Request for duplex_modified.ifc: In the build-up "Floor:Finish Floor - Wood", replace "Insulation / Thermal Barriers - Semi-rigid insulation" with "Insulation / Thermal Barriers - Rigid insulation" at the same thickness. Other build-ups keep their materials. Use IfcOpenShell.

First a look at what the model holds.

```python
import ifcopenshell
import ifcopenshell.util.element

model = ifcopenshell.open("duplex_modified.ifc")
print(model.schema)
for layer_set in model.by_type("IfcMaterialLayerSet"):
    if layer_set.LayerSetName == "Floor:Finish Floor - Wood":
        for layer in layer_set.MaterialLayers:
            print(layer.id(), layer.Material and layer.Material.Name, layer.LayerThickness, sep=" | ")
        print(len(ifcopenshell.util.element.get_elements_by_material(model, layer_set)), "elements and types use it")
print(sorted(m.Name for m in model.by_type("IfcMaterial") if m.Name)[:60])
```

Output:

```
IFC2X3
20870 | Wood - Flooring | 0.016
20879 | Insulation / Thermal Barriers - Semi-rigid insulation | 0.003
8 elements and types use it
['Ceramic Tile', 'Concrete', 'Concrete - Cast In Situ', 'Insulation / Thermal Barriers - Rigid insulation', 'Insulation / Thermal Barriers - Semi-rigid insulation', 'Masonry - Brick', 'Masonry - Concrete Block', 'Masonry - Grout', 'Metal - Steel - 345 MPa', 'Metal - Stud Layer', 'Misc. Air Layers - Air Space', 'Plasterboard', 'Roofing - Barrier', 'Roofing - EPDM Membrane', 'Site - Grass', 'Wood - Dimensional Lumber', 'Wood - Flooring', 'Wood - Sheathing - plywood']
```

```python
import ifcopenshell
import ifcopenshell.api.material

model = ifcopenshell.open("duplex_modified.ifc")

layer_set = next(s for s in model.by_type("IfcMaterialLayerSet") if s.LayerSetName == "Floor:Finish Floor - Wood")
layer = next(l for l in layer_set.MaterialLayers if l.Material and l.Material.Name == "Insulation / Thermal Barriers - Semi-rigid insulation")
material = next(m for m in model.by_type("IfcMaterial") if m.Name == "Insulation / Thermal Barriers - Rigid insulation")

# Point this one layer at the other material; renaming the old one would change it everywhere.
ifcopenshell.api.material.edit_layer(model, layer=layer, attributes={}, material=material)

print([l.Material.Name if l.Material else None for l in layer_set.MaterialLayers])

model.write("duplex_modified_edited.ifc")
```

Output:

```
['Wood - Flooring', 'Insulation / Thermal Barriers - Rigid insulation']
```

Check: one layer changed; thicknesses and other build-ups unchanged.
